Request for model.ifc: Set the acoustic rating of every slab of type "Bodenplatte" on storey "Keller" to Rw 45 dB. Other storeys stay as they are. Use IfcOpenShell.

First a look at what the model holds.

```python
import ifcopenshell
import ifcopenshell.util.element

model = ifcopenshell.open("model.ifc")
print(model.schema)
storey = next(s for s in model.by_type("IfcBuildingStorey") if s.Name == "Keller")
slabs = [e for e in ifcopenshell.util.element.get_decomposition(storey) if e.is_a("IfcSlab")]
seen = {}
for e in slabs:
    element_type = ifcopenshell.util.element.get_type(e)
    key = (element_type.Name if element_type != e and element_type else None, ifcopenshell.util.element.get_pset(e, "Pset_SlabCommon", "AcousticRating"))
    seen[key] = seen.get(key, 0) + 1
for (name, value), count in sorted(seen.items(), key=str):
    print(count, "x", name, "|", value)
```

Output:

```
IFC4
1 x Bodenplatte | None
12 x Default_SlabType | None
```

```python
import ifcopenshell
import ifcopenshell.api.pset
import ifcopenshell.util.element

model = ifcopenshell.open("model.ifc")

storey = next(s for s in model.by_type("IfcBuildingStorey") if s.Name == "Keller")
slabs = [e for e in ifcopenshell.util.element.get_decomposition(storey) if e.is_a("IfcSlab")]

count = 0
for e in slabs:
    element_type = ifcopenshell.util.element.get_type(e)
    if element_type in (None, e) or element_type.Name != "Bodenplatte":
        continue
    # add_pset returns the element's existing set when there is one.
    pset = ifcopenshell.api.pset.add_pset(model, product=e, name="Pset_SlabCommon")
    ifcopenshell.api.pset.edit_pset(model, pset=pset, properties={"AcousticRating": "Rw 45 dB"})
    count += 1

print(count, "slabs updated")

model.write("model-out.ifc")
```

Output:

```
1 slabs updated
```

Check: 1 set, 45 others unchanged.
